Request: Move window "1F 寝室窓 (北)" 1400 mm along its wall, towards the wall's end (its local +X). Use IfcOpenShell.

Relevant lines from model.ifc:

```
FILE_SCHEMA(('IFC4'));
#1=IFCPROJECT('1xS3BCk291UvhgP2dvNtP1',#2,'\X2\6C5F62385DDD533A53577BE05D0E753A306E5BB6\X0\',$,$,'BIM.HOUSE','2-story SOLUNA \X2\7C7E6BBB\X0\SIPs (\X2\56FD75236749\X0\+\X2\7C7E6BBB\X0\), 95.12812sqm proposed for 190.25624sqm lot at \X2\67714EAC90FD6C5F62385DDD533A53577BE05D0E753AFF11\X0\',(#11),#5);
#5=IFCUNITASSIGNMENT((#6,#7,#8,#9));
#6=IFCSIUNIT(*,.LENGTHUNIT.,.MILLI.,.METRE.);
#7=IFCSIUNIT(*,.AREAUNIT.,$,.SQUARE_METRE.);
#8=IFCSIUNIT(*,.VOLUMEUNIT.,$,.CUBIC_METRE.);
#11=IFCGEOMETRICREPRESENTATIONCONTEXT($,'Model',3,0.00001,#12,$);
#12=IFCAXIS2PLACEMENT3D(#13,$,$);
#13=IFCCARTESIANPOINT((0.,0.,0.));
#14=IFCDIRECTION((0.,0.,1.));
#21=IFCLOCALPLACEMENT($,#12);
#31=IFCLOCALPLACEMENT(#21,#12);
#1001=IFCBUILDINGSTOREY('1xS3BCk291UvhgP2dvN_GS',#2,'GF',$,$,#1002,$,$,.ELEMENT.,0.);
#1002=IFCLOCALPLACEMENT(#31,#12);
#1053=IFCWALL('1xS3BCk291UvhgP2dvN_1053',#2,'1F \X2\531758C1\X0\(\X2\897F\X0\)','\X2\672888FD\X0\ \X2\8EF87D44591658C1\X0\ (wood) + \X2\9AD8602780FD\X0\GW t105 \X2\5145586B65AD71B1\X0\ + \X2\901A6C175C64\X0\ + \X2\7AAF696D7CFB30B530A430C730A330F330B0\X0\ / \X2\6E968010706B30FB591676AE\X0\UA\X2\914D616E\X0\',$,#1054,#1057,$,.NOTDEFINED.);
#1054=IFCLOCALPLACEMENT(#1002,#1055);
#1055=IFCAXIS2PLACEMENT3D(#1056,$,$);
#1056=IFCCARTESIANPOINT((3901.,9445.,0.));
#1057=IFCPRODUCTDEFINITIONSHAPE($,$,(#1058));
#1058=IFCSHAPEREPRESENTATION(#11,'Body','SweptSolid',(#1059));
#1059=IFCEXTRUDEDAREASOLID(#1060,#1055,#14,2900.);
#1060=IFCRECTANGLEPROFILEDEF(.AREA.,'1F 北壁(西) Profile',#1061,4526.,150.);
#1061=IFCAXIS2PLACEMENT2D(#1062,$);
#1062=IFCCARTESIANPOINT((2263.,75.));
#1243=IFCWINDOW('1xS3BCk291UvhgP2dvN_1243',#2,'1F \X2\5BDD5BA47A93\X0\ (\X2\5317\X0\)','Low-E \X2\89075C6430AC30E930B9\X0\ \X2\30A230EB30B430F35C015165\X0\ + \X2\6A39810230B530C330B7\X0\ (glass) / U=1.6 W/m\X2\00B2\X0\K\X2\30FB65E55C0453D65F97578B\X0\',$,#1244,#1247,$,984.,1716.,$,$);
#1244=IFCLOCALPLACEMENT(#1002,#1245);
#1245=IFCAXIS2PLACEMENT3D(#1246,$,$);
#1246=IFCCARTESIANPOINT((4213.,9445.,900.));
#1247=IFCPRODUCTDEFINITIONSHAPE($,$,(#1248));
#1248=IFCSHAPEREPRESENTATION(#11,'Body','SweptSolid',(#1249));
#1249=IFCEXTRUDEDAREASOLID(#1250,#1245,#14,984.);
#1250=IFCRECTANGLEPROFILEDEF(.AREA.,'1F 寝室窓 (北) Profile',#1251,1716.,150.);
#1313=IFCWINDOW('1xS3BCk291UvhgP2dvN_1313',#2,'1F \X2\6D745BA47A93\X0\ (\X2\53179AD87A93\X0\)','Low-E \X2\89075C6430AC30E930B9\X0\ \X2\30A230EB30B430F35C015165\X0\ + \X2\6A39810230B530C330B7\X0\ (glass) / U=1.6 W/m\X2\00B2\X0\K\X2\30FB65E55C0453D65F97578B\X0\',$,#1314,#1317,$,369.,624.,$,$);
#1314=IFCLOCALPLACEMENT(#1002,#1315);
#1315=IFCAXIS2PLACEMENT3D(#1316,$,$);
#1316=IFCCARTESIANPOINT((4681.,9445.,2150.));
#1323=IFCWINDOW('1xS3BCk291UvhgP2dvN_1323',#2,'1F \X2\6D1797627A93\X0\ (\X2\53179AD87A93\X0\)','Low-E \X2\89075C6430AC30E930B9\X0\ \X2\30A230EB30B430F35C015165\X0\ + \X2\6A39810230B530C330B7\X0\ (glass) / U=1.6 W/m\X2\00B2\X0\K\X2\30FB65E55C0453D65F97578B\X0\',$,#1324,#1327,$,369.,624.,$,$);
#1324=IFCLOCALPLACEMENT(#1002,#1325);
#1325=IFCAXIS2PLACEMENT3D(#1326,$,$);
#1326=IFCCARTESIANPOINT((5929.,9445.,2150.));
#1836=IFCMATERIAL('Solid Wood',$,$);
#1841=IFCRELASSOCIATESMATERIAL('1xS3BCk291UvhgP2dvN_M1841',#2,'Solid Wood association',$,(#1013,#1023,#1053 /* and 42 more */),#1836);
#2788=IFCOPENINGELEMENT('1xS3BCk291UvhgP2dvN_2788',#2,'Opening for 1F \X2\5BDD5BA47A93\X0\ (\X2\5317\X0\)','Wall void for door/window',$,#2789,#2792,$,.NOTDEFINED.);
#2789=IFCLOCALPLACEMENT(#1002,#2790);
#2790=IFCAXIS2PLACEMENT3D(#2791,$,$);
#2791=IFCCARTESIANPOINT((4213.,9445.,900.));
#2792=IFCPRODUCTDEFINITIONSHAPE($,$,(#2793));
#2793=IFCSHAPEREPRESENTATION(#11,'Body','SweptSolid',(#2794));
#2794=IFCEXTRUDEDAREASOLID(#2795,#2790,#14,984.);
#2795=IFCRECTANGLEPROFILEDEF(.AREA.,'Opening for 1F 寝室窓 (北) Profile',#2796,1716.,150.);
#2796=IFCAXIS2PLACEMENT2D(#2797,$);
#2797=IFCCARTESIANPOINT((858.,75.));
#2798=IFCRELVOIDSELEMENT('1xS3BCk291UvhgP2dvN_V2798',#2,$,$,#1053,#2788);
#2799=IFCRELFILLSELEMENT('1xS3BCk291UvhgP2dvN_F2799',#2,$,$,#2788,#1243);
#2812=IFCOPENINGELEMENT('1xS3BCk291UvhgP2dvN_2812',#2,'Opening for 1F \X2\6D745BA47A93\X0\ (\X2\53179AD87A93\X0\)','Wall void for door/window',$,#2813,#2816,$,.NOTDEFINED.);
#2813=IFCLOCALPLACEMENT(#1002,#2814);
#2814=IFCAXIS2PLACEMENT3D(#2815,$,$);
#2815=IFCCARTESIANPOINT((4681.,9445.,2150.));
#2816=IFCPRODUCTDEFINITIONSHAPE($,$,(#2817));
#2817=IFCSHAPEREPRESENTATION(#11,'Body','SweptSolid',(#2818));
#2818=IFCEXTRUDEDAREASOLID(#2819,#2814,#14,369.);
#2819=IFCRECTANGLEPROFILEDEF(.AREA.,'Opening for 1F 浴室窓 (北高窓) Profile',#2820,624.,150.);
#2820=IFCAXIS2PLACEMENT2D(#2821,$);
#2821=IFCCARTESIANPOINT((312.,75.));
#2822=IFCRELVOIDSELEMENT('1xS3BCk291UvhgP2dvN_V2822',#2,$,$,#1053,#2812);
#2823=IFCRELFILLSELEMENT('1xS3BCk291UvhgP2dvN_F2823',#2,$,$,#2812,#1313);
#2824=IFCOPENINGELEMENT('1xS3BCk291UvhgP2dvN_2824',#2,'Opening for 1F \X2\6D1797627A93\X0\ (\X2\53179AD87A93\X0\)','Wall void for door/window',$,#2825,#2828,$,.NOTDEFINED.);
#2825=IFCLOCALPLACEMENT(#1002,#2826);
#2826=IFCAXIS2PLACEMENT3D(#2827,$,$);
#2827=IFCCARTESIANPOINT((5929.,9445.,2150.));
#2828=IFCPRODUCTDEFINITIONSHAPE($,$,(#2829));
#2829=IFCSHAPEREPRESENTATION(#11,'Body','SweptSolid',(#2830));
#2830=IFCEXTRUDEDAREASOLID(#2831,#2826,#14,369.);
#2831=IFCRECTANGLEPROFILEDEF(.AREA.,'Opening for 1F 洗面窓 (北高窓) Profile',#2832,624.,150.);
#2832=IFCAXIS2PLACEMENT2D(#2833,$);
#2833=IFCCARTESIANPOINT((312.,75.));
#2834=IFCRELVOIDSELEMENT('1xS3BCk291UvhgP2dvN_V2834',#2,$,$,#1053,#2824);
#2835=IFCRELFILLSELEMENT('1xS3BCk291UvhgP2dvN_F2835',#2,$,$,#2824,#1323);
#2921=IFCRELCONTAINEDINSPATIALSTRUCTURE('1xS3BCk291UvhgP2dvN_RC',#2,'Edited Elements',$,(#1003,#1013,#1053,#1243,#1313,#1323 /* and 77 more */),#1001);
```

```python
import ifcopenshell
import ifcopenshell.api.geometry
import ifcopenshell.util.placement
import ifcopenshell.util.unit

model = ifcopenshell.open("model.ifc")
unit_scale = ifcopenshell.util.unit.calculate_unit_scale(model)

window = model.by_guid("1xS3BCk291UvhgP2dvN_1243")
opening = window.FillsVoids[0].RelatingOpeningElement
wall = opening.VoidsElements[0].RelatingBuildingElement

wall_matrix = ifcopenshell.util.placement.get_local_placement(wall.ObjectPlacement)
shift = wall_matrix[:3, 0] * 1.4 / unit_scale
before = ifcopenshell.util.placement.get_local_placement(window.ObjectPlacement)[:3, 3].copy()

# The window is not placed relative to its opening, so move both.
for product in (opening, window):
    matrix = ifcopenshell.util.placement.get_local_placement(product.ObjectPlacement)
    matrix[:3, 3] += shift
    ifcopenshell.api.geometry.edit_object_placement(model, product=product, matrix=matrix, is_si=False)

after = ifcopenshell.util.placement.get_local_placement(window.ObjectPlacement)[:3, 3]
print("window moved by", (after - before).round(3) + 0.0)

model.write("model_v2.ifc")
```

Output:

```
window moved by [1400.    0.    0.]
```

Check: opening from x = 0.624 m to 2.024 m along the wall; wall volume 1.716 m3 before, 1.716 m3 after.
